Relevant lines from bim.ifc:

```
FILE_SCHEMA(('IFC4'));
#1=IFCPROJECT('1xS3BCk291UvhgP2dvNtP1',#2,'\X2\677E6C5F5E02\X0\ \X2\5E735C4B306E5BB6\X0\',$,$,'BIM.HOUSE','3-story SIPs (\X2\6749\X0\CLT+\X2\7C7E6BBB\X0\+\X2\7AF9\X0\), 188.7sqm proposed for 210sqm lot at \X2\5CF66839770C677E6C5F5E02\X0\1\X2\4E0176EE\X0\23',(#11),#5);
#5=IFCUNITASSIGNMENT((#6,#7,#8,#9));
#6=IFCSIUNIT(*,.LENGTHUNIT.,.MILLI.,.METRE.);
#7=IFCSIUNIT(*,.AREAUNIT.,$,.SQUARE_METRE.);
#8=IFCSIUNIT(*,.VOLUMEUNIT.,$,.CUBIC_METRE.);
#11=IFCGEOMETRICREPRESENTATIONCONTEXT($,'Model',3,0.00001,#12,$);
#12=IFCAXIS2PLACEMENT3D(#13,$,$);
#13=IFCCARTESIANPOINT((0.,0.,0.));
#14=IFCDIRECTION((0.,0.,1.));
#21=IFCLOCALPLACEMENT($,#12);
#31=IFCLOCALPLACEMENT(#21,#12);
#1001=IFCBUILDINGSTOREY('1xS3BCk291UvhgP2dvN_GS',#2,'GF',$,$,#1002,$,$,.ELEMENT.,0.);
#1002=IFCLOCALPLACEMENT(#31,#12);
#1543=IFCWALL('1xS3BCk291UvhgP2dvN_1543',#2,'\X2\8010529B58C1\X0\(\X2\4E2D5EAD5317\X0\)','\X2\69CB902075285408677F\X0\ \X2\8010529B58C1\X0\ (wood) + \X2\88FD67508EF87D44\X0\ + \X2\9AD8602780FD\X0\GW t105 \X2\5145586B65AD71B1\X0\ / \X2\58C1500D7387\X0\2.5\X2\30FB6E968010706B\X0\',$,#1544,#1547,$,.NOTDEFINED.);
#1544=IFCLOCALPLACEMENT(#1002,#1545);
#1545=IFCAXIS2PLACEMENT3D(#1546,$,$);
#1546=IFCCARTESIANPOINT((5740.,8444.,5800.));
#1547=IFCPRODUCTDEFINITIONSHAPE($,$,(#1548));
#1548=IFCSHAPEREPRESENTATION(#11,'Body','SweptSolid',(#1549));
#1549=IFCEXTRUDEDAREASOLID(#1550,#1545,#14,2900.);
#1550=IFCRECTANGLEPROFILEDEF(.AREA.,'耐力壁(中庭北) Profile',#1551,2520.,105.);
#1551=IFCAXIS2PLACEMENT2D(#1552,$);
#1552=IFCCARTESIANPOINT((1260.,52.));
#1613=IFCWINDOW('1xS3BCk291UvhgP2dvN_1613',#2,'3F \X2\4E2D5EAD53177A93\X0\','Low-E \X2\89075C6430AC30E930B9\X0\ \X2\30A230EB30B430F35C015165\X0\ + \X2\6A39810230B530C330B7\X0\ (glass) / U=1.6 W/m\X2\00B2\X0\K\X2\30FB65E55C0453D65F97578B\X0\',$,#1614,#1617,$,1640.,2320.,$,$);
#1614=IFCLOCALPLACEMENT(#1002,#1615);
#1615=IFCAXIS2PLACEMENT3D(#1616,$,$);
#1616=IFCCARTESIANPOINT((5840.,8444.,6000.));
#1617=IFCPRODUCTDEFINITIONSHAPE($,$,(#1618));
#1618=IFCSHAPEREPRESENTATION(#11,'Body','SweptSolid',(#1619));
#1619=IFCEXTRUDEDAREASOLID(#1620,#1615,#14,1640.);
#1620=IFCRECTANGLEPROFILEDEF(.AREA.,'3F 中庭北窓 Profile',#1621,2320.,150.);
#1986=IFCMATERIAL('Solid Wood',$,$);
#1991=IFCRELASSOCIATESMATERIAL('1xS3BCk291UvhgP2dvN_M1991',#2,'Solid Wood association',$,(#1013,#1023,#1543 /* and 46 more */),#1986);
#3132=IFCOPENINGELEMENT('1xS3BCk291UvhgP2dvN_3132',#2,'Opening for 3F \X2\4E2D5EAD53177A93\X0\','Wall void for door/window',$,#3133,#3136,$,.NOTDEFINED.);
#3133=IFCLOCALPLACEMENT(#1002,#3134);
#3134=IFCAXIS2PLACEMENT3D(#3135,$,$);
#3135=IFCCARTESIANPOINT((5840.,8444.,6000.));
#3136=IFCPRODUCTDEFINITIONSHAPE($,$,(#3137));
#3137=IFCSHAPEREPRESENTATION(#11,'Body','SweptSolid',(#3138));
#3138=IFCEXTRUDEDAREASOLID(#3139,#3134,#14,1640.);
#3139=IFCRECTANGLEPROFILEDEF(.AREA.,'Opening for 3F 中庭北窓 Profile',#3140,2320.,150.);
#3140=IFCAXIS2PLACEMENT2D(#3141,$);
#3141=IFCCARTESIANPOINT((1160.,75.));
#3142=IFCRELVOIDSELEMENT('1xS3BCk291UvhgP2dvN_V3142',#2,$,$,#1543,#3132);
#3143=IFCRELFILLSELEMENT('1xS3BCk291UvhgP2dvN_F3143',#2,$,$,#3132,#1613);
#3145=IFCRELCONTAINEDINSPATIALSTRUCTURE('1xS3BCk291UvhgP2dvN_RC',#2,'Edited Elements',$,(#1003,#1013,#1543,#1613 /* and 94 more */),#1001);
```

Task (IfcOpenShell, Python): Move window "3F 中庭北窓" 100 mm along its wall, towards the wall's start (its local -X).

```python
import ifcopenshell
import ifcopenshell.api.geometry
import ifcopenshell.util.placement
import ifcopenshell.util.unit

model = ifcopenshell.open("bim.ifc")
unit_scale = ifcopenshell.util.unit.calculate_unit_scale(model)

window = model.by_guid("1xS3BCk291UvhgP2dvN_1613")
opening = window.FillsVoids[0].RelatingOpeningElement
wall = opening.VoidsElements[0].RelatingBuildingElement

wall_matrix = ifcopenshell.util.placement.get_local_placement(wall.ObjectPlacement)
shift = wall_matrix[:3, 0] * -0.1 / unit_scale
before = ifcopenshell.util.placement.get_local_placement(window.ObjectPlacement)[:3, 3].copy()

# The window is not placed relative to its opening, so move both.
for product in (opening, window):
    matrix = ifcopenshell.util.placement.get_local_placement(product.ObjectPlacement)
    matrix[:3, 3] += shift
    ifcopenshell.api.geometry.edit_object_placement(model, product=product, matrix=matrix, is_si=False)

after = ifcopenshell.util.placement.get_local_placement(window.ObjectPlacement)[:3, 3]
print("window moved by", (after - before).round(3) + 0.0)

model.write("bim_edited.ifc")
```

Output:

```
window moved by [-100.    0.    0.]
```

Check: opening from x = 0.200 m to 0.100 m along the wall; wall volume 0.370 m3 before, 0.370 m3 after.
